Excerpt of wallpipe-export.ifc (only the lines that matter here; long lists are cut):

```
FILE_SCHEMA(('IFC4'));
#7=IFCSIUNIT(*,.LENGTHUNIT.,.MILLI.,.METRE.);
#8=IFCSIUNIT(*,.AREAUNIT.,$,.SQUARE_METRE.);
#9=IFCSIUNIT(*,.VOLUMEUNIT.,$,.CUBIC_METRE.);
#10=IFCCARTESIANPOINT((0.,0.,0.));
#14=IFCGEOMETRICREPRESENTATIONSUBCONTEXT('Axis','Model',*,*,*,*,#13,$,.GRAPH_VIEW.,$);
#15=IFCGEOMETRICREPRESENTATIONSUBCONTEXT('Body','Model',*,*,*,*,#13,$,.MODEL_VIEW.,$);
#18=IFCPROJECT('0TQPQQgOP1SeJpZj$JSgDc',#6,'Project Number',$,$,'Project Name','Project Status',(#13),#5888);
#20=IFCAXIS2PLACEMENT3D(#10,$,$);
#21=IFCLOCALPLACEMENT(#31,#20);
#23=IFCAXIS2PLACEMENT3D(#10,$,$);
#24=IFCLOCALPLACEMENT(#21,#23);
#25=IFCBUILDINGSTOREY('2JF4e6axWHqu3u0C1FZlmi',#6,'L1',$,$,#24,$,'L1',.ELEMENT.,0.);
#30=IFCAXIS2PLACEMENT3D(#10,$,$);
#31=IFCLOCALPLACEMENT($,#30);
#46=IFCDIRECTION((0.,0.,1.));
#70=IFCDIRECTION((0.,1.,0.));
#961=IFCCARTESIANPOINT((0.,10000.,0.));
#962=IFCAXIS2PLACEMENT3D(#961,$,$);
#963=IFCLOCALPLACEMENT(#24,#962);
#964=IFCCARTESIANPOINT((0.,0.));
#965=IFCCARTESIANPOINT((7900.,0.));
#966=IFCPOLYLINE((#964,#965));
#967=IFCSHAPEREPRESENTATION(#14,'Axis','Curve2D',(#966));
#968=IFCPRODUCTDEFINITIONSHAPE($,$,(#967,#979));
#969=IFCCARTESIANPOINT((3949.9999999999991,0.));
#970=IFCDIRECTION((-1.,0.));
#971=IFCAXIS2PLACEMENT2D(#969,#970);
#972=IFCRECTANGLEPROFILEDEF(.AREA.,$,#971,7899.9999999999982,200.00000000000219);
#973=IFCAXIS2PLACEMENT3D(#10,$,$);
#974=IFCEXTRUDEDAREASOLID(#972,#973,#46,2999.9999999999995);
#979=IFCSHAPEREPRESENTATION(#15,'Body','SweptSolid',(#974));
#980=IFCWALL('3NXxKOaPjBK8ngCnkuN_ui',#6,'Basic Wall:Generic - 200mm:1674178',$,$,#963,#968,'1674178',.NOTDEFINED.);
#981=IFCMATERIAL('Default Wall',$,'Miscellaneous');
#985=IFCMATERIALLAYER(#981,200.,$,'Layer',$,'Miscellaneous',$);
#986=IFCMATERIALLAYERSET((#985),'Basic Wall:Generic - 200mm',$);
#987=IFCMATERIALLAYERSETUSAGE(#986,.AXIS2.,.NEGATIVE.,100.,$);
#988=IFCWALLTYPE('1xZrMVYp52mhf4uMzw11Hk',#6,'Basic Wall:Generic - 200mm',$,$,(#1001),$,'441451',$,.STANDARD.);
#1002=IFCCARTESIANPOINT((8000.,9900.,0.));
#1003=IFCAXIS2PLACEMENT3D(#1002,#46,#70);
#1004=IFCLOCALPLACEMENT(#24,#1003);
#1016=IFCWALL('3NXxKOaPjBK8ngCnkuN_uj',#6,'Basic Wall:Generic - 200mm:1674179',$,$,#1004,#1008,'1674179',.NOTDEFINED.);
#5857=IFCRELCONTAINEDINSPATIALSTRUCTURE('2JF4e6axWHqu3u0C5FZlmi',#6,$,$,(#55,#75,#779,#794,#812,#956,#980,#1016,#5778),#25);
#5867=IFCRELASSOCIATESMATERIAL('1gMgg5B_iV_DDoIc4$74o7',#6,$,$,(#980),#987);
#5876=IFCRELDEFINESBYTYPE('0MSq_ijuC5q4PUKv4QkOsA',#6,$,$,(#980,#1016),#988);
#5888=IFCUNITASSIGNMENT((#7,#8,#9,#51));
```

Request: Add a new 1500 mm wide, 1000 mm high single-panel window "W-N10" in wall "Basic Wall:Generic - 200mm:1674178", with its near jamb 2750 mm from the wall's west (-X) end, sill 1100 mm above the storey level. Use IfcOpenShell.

```python
import numpy as np
import ifcopenshell
import ifcopenshell.api.feature
import ifcopenshell.api.geometry
import ifcopenshell.api.root
import ifcopenshell.api.spatial
import ifcopenshell.geom
import ifcopenshell.util.element
import ifcopenshell.util.placement
import ifcopenshell.util.representation
import ifcopenshell.util.shape
import ifcopenshell.util.unit

model = ifcopenshell.open("wallpipe-export.ifc")
unit_scale = ifcopenshell.util.unit.calculate_unit_scale(model)
settings = ifcopenshell.geom.settings()


def volume(element):
    """Net volume in cubic metres, openings subtracted."""
    shape = ifcopenshell.geom.create_shape(settings, element)
    return ifcopenshell.util.shape.get_volume(shape.geometry)


wall = model.by_guid("3NXxKOaPjBK8ngCnkuN_ui")
storey = ifcopenshell.util.element.get_container(wall, ifc_class="IfcBuildingStorey")
context = ifcopenshell.util.representation.get_context(model, "Model", "Body", "MODEL_VIEW")
before = volume(wall)

width, height, from_end, sill = 1.5, 1, 2.75, 1.1  # metres

# The wall runs along its own X axis, and the end named is its -X end.
wall_shape = ifcopenshell.geom.create_shape(settings, wall)
x, y, z = ifcopenshell.util.shape.get_vertices(wall_shape.geometry).T
start = x.min() + from_end
face, thickness = float(y.min()), float(y.max() - y.min())
wall_matrix = ifcopenshell.util.placement.get_local_placement(wall.ObjectPlacement)
level = ifcopenshell.util.placement.get_local_placement(storey.ObjectPlacement)[2, 3]


def in_wall(x, y):
    """Placement at x, y metres in the wall's axes, at sill height."""
    matrix = wall_matrix.copy()
    matrix[:, 3] = wall_matrix @ np.array([x / unit_scale, y / unit_scale, 0.0, 1.0])
    matrix[2, 3] = level + sill / unit_scale
    return matrix


# Opening: a box that overshoots both wall faces by 50 mm.
opening = ifcopenshell.api.root.create_entity(model, ifc_class="IfcOpeningElement", predefined_type="OPENING")
box = ifcopenshell.api.geometry.add_wall_representation(
    model, context=context, length=width, height=height, thickness=thickness + 0.1
)
ifcopenshell.api.geometry.assign_representation(model, product=opening, representation=box)
ifcopenshell.api.geometry.edit_object_placement(model, product=opening, matrix=in_wall(start, face - 0.05), is_si=False)
ifcopenshell.api.feature.add_feature(model, feature=opening, element=wall)

window = ifcopenshell.api.root.create_entity(model, ifc_class="IfcWindow", name="W-N10", predefined_type="WINDOW")
window.OverallWidth, window.OverallHeight = width / unit_scale, height / unit_scale
window.PartitioningType = "SINGLE_PANEL"
body = ifcopenshell.api.geometry.add_window_representation(
    model,
    context=context,
    overall_width=window.OverallWidth,
    overall_height=window.OverallHeight,
    partition_type="SINGLE_PANEL",
)
ifcopenshell.api.geometry.assign_representation(model, product=window, representation=body)
ifcopenshell.api.spatial.assign_container(model, products=[window], relating_structure=storey)
ifcopenshell.api.feature.add_filling(model, opening=opening, element=window)

# Centre the window in the wall's thickness.
ifcopenshell.api.geometry.edit_object_placement(model, product=window, matrix=in_wall(start, face), is_si=False)
window_shape = ifcopenshell.geom.create_shape(settings, window)
depth = ifcopenshell.util.shape.get_vertices(window_shape.geometry)[:, 1]
offset = face + thickness / 2 - (depth.min() + depth.max()) / 2
ifcopenshell.api.geometry.edit_object_placement(model, product=window, matrix=in_wall(start, offset), is_si=False)

after = volume(wall)

print(f"wall volume {before:.3f} -> {after:.3f} m3")

model.write("wallpipe-export_v2.ifc")
```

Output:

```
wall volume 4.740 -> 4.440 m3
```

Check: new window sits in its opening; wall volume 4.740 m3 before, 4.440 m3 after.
